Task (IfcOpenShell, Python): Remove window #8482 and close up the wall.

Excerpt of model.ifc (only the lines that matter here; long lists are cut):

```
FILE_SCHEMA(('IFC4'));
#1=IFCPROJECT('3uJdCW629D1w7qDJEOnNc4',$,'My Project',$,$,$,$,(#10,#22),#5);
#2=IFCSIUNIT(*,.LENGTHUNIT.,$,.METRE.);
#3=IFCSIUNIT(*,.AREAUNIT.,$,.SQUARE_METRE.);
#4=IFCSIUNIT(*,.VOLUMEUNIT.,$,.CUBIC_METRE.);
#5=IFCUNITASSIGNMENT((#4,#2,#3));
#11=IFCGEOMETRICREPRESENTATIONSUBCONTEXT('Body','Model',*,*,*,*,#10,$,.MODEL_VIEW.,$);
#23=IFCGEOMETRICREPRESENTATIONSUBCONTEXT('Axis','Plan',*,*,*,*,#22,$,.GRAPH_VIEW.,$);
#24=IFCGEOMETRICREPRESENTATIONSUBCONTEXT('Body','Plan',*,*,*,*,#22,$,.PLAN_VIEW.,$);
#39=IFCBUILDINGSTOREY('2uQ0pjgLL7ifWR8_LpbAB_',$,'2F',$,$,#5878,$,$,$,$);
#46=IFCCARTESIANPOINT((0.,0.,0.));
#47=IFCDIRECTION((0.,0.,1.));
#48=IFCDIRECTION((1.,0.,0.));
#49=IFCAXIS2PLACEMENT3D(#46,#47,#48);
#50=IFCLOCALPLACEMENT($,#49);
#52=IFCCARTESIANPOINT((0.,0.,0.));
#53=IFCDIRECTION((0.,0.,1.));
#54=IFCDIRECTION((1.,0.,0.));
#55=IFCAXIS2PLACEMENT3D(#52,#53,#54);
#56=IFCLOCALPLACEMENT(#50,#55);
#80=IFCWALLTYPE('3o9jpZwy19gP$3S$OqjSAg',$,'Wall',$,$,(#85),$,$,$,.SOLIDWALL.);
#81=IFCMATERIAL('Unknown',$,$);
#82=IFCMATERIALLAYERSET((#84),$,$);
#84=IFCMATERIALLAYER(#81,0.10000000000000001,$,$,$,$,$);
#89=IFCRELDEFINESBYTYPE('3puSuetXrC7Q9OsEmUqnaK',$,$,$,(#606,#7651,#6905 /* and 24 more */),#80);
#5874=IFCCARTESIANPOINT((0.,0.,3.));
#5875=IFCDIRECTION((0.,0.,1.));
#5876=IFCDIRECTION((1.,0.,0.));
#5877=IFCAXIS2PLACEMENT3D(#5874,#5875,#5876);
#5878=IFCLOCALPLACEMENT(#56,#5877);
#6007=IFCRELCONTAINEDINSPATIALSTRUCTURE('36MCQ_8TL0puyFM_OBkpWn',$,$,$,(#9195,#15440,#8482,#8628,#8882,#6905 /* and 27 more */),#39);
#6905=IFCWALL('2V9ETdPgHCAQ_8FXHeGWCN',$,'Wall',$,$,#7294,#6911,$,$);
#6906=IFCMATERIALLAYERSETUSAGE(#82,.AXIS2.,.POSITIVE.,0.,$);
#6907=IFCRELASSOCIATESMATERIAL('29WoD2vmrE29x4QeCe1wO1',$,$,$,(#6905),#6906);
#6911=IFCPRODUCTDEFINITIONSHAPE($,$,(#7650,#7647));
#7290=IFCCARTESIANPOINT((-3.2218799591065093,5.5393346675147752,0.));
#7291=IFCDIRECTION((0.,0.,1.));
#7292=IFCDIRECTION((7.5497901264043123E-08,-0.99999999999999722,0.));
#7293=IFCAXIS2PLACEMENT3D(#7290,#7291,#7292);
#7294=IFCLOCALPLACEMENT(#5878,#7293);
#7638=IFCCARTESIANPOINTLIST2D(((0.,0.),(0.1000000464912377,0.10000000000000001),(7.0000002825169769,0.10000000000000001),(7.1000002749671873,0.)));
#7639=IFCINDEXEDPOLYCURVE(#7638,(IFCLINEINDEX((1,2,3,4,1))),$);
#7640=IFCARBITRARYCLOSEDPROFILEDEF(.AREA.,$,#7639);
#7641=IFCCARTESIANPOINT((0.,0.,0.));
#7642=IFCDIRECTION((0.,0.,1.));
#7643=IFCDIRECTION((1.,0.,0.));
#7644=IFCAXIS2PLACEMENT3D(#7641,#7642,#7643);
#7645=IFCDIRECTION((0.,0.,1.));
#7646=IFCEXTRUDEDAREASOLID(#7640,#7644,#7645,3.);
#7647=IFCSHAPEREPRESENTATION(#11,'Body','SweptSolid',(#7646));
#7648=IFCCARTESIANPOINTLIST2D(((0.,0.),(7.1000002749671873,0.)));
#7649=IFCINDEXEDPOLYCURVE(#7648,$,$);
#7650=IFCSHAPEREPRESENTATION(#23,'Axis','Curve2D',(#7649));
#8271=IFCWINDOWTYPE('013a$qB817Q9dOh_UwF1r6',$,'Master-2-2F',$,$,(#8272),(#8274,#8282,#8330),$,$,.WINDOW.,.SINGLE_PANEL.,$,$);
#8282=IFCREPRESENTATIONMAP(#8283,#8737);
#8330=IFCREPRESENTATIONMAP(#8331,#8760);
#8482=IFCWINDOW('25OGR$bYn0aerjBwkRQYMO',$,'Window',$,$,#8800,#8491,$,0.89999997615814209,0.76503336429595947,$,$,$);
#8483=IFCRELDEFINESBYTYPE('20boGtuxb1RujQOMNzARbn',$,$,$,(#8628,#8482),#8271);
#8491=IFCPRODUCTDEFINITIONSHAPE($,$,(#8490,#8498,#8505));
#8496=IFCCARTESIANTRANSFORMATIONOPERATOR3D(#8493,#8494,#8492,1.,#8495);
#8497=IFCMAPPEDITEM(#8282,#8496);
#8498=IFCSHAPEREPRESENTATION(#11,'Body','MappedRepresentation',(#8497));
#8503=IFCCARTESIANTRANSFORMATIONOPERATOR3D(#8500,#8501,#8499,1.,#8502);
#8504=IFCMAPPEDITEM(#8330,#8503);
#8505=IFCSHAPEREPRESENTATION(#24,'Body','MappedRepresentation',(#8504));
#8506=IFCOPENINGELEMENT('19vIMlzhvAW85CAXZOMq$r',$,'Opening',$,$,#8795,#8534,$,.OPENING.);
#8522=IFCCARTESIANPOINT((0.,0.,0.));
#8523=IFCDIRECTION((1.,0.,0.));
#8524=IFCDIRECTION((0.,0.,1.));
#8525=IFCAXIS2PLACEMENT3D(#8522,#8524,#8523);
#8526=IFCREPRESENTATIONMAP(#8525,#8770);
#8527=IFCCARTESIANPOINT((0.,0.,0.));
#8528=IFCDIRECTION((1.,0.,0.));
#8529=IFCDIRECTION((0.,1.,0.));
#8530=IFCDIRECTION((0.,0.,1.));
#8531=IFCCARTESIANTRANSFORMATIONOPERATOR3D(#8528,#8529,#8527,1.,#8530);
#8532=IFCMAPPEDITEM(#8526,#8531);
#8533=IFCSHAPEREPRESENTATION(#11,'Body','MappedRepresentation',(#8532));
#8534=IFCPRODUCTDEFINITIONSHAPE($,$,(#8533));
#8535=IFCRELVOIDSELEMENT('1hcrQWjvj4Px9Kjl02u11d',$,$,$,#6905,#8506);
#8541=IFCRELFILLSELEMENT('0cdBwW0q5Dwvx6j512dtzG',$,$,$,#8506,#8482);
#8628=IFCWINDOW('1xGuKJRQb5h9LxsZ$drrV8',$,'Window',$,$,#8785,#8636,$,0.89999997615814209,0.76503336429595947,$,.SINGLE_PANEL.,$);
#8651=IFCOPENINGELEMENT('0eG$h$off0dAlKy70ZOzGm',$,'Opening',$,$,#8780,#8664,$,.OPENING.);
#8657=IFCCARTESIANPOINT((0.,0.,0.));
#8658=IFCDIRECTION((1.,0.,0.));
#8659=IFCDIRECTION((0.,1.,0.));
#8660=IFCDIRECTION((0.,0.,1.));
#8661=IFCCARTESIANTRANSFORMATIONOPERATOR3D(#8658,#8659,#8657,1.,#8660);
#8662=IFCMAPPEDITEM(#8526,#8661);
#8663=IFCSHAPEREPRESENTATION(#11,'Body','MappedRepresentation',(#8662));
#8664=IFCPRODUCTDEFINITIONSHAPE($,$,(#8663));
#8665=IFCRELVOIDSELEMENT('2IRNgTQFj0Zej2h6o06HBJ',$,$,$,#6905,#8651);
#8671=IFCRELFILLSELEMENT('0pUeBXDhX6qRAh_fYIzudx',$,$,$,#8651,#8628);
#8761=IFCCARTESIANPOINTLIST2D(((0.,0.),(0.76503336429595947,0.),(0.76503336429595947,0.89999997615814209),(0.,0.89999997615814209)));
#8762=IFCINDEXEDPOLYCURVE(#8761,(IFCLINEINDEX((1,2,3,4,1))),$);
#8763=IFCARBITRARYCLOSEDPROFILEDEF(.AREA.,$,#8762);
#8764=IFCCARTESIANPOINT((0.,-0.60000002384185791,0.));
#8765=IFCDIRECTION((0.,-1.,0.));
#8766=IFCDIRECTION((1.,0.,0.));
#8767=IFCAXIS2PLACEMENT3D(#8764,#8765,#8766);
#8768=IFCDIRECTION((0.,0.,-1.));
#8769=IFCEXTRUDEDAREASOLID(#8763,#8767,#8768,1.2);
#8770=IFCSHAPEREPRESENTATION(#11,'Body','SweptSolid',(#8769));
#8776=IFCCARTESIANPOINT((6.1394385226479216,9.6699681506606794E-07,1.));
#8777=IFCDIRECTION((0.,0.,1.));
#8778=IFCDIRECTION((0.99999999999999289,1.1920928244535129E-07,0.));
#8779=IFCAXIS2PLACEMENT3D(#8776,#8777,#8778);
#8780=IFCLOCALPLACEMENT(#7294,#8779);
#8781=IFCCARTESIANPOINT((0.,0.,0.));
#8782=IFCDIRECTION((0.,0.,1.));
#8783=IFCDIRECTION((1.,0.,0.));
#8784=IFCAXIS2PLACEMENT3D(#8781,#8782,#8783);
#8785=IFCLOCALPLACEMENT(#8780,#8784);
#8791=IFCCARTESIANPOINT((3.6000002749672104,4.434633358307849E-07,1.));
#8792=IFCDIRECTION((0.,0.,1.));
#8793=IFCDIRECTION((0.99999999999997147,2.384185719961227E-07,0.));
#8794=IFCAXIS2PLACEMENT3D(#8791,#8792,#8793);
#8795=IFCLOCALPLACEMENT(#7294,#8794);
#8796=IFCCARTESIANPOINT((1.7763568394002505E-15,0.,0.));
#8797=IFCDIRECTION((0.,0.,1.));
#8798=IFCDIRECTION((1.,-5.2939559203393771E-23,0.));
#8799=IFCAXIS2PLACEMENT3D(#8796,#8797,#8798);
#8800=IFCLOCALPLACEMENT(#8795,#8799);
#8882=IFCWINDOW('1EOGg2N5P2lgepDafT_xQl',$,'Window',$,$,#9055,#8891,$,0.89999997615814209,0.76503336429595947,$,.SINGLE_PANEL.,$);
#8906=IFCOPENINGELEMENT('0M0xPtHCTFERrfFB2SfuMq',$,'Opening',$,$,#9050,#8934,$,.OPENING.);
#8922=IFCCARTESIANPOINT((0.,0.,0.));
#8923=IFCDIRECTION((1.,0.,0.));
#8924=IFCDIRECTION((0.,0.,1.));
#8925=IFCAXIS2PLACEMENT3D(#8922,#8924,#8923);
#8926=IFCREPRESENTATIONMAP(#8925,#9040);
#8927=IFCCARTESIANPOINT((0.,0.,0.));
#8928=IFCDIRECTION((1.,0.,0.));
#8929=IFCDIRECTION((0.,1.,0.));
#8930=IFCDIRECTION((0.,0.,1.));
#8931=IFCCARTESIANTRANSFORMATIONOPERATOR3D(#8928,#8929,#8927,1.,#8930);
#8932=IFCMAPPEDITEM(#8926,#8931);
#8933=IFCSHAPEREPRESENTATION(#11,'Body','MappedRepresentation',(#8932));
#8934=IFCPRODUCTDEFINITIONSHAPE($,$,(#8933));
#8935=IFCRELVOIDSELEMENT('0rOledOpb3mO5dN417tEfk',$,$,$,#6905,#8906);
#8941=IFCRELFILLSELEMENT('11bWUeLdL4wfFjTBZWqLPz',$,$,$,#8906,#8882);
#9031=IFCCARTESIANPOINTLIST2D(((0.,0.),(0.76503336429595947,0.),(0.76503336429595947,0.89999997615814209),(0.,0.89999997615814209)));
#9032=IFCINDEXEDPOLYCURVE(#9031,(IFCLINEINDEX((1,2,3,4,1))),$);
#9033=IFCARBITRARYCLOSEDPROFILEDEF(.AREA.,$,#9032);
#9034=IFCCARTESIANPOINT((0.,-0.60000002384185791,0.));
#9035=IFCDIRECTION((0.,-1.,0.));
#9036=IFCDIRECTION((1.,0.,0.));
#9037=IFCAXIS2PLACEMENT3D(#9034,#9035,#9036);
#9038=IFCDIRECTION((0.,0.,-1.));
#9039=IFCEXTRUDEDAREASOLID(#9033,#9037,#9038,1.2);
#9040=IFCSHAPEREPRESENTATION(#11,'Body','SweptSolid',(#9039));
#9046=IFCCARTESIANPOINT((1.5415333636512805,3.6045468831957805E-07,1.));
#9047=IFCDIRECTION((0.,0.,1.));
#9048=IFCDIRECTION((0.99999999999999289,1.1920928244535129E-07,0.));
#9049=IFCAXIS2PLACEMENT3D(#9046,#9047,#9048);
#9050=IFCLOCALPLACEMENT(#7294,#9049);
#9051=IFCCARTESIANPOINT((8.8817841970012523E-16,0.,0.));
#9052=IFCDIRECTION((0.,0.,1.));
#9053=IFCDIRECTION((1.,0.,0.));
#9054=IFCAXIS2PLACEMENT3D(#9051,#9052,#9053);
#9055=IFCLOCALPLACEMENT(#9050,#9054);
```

```python
import ifcopenshell
import ifcopenshell.api.feature
import ifcopenshell.api.root
import ifcopenshell.geom
import ifcopenshell.util.shape

model = ifcopenshell.open("model.ifc")
settings = ifcopenshell.geom.settings()


def volume(element):
    """Net volume in cubic metres, openings subtracted."""
    shape = ifcopenshell.geom.create_shape(settings, element)
    return ifcopenshell.util.shape.get_volume(shape.geometry)


window = model.by_guid("25OGR$bYn0aerjBwkRQYMO")
opening = window.FillsVoids[0].RelatingOpeningElement
wall = opening.VoidsElements[0].RelatingBuildingElement
before = volume(wall)

ifcopenshell.api.root.remove_product(model, product=window)
ifcopenshell.api.feature.remove_feature(model, feature=opening)

after = volume(wall)

print(f"wall volume {before:.3f} -> {after:.3f} m3")

model.write("model_edited.ifc")
```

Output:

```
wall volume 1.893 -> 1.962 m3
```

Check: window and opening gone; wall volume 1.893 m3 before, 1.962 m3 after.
